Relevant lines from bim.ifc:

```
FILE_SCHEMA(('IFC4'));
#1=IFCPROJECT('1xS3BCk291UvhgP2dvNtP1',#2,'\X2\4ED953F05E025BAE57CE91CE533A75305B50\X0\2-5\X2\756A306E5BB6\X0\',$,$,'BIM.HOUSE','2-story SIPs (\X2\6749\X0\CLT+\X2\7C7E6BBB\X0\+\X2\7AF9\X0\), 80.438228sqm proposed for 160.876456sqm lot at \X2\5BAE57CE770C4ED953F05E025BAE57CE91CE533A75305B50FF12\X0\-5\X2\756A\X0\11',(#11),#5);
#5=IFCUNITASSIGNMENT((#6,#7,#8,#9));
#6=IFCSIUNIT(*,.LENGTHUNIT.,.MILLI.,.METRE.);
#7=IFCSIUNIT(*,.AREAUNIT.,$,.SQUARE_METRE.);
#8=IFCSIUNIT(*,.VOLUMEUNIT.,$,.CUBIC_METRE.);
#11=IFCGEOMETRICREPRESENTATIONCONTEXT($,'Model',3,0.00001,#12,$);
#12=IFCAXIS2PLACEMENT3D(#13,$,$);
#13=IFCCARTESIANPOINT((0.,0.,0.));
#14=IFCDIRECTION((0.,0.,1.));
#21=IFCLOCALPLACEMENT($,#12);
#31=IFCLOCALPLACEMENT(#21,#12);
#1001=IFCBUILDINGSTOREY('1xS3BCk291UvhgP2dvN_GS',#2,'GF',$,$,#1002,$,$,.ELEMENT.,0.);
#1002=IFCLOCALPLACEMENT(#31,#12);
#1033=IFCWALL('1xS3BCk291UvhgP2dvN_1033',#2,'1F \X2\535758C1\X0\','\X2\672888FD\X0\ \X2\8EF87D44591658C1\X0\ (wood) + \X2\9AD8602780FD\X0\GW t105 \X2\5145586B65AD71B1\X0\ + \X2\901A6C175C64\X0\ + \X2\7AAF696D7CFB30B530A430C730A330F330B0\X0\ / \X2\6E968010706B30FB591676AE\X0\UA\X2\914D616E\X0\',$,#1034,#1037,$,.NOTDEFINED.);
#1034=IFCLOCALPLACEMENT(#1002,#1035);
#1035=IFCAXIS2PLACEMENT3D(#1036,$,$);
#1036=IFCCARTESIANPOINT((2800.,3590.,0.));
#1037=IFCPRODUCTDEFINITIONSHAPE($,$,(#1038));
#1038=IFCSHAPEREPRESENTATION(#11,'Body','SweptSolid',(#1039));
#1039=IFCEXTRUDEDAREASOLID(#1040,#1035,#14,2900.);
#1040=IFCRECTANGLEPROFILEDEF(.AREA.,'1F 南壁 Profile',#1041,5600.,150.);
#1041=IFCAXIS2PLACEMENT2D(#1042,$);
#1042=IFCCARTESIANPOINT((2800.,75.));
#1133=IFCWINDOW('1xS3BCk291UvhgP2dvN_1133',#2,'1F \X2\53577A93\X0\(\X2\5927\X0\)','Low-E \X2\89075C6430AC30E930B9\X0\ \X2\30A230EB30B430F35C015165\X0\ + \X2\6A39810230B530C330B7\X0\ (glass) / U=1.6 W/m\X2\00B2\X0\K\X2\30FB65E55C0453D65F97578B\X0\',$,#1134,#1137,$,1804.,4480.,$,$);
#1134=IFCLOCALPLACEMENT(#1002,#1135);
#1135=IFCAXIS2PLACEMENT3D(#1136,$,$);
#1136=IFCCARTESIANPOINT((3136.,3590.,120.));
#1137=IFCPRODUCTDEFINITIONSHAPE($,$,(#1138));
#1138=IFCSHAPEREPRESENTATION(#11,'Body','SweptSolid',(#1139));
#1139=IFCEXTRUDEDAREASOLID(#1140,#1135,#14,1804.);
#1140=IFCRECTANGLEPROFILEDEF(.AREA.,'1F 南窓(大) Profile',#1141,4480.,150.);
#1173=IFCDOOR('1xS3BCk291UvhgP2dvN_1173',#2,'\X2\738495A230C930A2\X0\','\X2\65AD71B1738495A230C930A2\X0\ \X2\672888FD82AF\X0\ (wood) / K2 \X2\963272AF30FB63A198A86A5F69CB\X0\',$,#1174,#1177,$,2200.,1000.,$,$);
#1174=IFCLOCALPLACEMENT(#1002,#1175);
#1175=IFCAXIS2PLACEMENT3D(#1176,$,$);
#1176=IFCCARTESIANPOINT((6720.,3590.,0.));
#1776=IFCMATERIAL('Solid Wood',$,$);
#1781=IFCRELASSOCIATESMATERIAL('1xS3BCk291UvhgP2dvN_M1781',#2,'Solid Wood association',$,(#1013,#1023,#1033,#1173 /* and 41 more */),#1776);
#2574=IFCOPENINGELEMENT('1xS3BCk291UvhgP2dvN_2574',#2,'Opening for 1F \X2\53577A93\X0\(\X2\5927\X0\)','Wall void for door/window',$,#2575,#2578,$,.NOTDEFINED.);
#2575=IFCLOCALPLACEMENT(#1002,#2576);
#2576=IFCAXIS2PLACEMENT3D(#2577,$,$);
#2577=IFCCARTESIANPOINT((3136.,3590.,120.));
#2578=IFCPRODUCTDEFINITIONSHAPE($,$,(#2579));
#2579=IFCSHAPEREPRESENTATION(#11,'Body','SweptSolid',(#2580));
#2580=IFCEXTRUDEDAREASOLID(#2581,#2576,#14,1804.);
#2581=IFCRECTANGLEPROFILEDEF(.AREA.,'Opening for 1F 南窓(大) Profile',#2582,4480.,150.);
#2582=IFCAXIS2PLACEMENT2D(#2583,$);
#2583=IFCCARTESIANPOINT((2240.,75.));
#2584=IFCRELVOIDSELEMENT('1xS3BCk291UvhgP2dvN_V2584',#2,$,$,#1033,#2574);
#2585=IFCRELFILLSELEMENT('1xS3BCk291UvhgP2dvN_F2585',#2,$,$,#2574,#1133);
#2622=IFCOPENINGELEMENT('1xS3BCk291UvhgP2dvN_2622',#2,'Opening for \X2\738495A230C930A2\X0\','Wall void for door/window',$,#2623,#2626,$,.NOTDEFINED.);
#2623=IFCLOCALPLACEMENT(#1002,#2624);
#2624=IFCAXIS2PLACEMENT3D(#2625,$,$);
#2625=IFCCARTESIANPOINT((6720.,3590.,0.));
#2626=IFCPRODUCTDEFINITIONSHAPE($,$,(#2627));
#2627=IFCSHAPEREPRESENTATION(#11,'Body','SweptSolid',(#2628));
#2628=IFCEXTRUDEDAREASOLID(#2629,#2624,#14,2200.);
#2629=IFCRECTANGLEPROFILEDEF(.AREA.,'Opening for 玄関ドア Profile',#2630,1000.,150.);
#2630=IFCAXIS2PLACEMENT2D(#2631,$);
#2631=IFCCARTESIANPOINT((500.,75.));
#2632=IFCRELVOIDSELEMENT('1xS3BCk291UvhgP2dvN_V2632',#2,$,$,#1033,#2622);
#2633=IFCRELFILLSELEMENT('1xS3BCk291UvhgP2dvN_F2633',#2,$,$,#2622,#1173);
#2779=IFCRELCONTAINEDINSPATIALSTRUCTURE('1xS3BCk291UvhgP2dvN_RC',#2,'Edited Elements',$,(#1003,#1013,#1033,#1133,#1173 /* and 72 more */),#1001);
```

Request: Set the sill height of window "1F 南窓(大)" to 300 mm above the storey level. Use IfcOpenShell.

```python
import numpy as np
import ifcopenshell
import ifcopenshell.api.geometry
import ifcopenshell.geom
import ifcopenshell.util.element
import ifcopenshell.util.placement
import ifcopenshell.util.shape
import ifcopenshell.util.unit

model = ifcopenshell.open("bim.ifc")
unit_scale = ifcopenshell.util.unit.calculate_unit_scale(model)

window = model.by_id(1133)
opening = window.FillsVoids[0].RelatingOpeningElement
storey = ifcopenshell.util.element.get_container(window, ifc_class="IfcBuildingStorey")
level = ifcopenshell.util.placement.get_local_placement(storey.ObjectPlacement)[2, 3]

# The opening's origin need not be at the sill, so measure its lowest point.
shape = ifcopenshell.geom.create_shape(ifcopenshell.geom.settings(), opening)
bottom = ifcopenshell.util.shape.get_shape_bottom_elevation(shape, shape.geometry) / unit_scale
dz = level + 300.0 - bottom

shift = np.array([0.0, 0.0, dz])
# The window is not placed relative to its opening, so move both.
for product in (opening, window):
    matrix = ifcopenshell.util.placement.get_local_placement(product.ObjectPlacement)
    matrix[:3, 3] += shift
    ifcopenshell.api.geometry.edit_object_placement(model, product=product, matrix=matrix, is_si=False)

print(f"moved by {dz * unit_scale:+.3f} m")

model.write("bim_updated.ifc")
```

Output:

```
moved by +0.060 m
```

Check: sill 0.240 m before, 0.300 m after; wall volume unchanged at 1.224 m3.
